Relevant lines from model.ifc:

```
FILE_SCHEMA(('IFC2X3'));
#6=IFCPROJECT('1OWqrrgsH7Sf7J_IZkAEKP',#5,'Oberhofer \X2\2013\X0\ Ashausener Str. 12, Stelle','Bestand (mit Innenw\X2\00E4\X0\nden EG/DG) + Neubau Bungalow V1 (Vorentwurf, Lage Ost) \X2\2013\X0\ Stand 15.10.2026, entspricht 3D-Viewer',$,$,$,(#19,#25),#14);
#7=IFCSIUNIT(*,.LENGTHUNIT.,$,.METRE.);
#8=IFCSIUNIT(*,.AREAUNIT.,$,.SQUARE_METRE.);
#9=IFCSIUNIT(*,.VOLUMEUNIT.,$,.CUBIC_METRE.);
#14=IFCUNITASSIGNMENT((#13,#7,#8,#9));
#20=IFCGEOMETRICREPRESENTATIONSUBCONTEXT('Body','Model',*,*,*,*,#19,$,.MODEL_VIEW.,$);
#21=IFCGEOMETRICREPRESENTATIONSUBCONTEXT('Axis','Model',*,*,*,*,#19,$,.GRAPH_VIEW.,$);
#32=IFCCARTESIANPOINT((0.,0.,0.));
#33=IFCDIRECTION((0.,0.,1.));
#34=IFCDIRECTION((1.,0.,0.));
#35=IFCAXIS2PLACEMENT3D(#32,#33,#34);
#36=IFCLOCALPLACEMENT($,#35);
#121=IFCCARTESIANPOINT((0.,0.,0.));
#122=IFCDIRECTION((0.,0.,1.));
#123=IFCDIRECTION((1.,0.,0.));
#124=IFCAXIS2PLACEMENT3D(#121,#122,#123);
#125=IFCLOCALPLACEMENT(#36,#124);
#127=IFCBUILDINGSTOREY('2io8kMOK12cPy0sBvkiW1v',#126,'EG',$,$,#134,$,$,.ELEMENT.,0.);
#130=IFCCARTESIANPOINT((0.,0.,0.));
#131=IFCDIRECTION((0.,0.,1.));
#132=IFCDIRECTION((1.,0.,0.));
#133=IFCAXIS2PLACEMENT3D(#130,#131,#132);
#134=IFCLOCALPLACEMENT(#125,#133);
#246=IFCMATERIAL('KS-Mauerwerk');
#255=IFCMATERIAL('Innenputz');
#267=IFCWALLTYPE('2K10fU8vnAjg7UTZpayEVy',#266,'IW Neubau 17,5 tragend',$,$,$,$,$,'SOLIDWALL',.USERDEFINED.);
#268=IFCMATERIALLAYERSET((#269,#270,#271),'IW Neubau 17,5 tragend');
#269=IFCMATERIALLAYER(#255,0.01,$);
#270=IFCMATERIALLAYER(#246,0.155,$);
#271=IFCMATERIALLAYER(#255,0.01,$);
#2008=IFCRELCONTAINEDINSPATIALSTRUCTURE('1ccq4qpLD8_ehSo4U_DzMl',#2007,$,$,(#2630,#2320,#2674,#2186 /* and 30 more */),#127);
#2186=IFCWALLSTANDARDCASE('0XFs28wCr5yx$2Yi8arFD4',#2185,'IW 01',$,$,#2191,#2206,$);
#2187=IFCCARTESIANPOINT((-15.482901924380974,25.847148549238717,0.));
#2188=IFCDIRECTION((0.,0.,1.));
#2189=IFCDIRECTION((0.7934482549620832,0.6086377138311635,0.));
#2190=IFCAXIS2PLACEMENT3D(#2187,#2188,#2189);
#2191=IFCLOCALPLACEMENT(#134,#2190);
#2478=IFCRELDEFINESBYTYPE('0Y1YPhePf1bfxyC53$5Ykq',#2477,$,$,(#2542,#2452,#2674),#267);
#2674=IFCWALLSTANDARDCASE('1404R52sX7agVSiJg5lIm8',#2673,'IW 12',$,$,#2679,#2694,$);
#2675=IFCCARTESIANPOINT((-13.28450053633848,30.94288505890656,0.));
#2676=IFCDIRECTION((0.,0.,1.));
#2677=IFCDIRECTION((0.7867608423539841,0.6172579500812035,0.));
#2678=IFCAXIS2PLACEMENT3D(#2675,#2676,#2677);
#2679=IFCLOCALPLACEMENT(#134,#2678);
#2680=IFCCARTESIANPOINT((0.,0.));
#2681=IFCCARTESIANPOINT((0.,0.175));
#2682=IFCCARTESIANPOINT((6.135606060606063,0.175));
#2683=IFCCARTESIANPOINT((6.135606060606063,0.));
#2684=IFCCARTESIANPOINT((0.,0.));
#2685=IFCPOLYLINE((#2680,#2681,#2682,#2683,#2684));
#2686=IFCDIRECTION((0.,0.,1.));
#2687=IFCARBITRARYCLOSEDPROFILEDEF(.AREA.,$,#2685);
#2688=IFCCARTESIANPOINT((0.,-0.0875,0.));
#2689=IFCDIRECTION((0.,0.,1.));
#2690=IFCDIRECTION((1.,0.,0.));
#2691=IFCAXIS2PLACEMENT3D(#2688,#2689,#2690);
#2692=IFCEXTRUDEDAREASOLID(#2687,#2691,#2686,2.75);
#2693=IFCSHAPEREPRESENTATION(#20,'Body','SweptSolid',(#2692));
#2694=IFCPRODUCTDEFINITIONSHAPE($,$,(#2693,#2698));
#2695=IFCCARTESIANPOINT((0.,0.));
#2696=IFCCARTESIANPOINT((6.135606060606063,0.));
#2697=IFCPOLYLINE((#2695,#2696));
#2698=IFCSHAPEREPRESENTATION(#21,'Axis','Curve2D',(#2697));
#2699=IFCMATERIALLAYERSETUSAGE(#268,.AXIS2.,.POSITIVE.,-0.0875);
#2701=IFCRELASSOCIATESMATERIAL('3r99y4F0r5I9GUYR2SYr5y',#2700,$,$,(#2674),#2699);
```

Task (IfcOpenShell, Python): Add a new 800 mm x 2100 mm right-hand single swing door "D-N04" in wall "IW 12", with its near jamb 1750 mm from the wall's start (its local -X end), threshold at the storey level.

```python
import numpy as np
import ifcopenshell
import ifcopenshell.api.feature
import ifcopenshell.api.geometry
import ifcopenshell.api.root
import ifcopenshell.api.spatial
import ifcopenshell.api.type
import ifcopenshell.geom
import ifcopenshell.util.element
import ifcopenshell.util.placement
import ifcopenshell.util.representation
import ifcopenshell.util.shape
import ifcopenshell.util.unit

model = ifcopenshell.open("model.ifc")
unit_scale = ifcopenshell.util.unit.calculate_unit_scale(model)
settings = ifcopenshell.geom.settings()


def volume(element):
    """Net volume in cubic metres, openings subtracted."""
    shape = ifcopenshell.geom.create_shape(settings, element)
    return ifcopenshell.util.shape.get_volume(shape.geometry)


wall = model.by_id(2674)
storey = ifcopenshell.util.element.get_container(wall, ifc_class="IfcBuildingStorey")
context = ifcopenshell.util.representation.get_context(model, "Model", "Body", "MODEL_VIEW")
before = volume(wall)

width, height, from_end, sill = 0.8, 2.1, 1.75, 0.0  # metres

# The wall runs along its own X axis, and the end named is its -X end.
wall_shape = ifcopenshell.geom.create_shape(settings, wall)
x, y, z = ifcopenshell.util.shape.get_vertices(wall_shape.geometry).T
start = x.min() + from_end
face, thickness = float(y.min()), float(y.max() - y.min())
wall_matrix = ifcopenshell.util.placement.get_local_placement(wall.ObjectPlacement)
level = ifcopenshell.util.placement.get_local_placement(storey.ObjectPlacement)[2, 3]


def in_wall(x, y):
    """Placement at x, y metres in the wall's axes, at sill height."""
    matrix = wall_matrix.copy()
    matrix[:, 3] = wall_matrix @ np.array([x / unit_scale, y / unit_scale, 0.0, 1.0])
    matrix[2, 3] = level + sill / unit_scale
    return matrix


# Opening: a box that overshoots both wall faces by 50 mm.
opening = ifcopenshell.api.root.create_entity(model, ifc_class="IfcOpeningElement")
box = ifcopenshell.api.geometry.add_wall_representation(
    model, context=context, length=width, height=height, thickness=thickness + 0.1
)
ifcopenshell.api.geometry.assign_representation(model, product=opening, representation=box)
ifcopenshell.api.geometry.edit_object_placement(model, product=opening, matrix=in_wall(start, face - 0.05), is_si=False)
ifcopenshell.api.feature.add_feature(model, feature=opening, element=wall)

door = ifcopenshell.api.root.create_entity(model, ifc_class="IfcDoor", name="D-N04")
door.OverallWidth, door.OverallHeight = width / unit_scale, height / unit_scale
body = ifcopenshell.api.geometry.add_door_representation(
    model,
    context=context,
    overall_width=door.OverallWidth,
    overall_height=door.OverallHeight,
    operation_type="SINGLE_SWING_RIGHT",
    lining_properties={"LiningDepth": thickness / unit_scale, "ThresholdDepth": thickness / unit_scale},
)
ifcopenshell.api.geometry.assign_representation(model, product=door, representation=body)
ifcopenshell.api.spatial.assign_container(model, products=[door], relating_structure=storey)
fills = ifcopenshell.api.feature.add_filling(model, opening=opening, element=door)
fills.OwnerHistory = door.OwnerHistory  # required in IFC2X3

# IFC2X3 keeps the operation on the door style.
style = ifcopenshell.api.root.create_entity(model, ifc_class="IfcDoorStyle", name="D-N04")
style.OperationType, style.ConstructionType = "SINGLE_SWING_RIGHT", "NOTDEFINED"
style.ParameterTakesPrecedence = style.Sizeable = False
ifcopenshell.api.type.assign_type(model, related_objects=[door], relating_type=style)

# The lining spans the wall, so the door starts at the wall face.
ifcopenshell.api.geometry.edit_object_placement(model, product=door, matrix=in_wall(start, face), is_si=False)

after = volume(wall)

print(f"wall volume {before:.3f} -> {after:.3f} m3")

model.write("model_rev.ifc")
```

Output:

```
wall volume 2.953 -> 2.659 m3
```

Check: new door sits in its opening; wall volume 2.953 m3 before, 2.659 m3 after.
